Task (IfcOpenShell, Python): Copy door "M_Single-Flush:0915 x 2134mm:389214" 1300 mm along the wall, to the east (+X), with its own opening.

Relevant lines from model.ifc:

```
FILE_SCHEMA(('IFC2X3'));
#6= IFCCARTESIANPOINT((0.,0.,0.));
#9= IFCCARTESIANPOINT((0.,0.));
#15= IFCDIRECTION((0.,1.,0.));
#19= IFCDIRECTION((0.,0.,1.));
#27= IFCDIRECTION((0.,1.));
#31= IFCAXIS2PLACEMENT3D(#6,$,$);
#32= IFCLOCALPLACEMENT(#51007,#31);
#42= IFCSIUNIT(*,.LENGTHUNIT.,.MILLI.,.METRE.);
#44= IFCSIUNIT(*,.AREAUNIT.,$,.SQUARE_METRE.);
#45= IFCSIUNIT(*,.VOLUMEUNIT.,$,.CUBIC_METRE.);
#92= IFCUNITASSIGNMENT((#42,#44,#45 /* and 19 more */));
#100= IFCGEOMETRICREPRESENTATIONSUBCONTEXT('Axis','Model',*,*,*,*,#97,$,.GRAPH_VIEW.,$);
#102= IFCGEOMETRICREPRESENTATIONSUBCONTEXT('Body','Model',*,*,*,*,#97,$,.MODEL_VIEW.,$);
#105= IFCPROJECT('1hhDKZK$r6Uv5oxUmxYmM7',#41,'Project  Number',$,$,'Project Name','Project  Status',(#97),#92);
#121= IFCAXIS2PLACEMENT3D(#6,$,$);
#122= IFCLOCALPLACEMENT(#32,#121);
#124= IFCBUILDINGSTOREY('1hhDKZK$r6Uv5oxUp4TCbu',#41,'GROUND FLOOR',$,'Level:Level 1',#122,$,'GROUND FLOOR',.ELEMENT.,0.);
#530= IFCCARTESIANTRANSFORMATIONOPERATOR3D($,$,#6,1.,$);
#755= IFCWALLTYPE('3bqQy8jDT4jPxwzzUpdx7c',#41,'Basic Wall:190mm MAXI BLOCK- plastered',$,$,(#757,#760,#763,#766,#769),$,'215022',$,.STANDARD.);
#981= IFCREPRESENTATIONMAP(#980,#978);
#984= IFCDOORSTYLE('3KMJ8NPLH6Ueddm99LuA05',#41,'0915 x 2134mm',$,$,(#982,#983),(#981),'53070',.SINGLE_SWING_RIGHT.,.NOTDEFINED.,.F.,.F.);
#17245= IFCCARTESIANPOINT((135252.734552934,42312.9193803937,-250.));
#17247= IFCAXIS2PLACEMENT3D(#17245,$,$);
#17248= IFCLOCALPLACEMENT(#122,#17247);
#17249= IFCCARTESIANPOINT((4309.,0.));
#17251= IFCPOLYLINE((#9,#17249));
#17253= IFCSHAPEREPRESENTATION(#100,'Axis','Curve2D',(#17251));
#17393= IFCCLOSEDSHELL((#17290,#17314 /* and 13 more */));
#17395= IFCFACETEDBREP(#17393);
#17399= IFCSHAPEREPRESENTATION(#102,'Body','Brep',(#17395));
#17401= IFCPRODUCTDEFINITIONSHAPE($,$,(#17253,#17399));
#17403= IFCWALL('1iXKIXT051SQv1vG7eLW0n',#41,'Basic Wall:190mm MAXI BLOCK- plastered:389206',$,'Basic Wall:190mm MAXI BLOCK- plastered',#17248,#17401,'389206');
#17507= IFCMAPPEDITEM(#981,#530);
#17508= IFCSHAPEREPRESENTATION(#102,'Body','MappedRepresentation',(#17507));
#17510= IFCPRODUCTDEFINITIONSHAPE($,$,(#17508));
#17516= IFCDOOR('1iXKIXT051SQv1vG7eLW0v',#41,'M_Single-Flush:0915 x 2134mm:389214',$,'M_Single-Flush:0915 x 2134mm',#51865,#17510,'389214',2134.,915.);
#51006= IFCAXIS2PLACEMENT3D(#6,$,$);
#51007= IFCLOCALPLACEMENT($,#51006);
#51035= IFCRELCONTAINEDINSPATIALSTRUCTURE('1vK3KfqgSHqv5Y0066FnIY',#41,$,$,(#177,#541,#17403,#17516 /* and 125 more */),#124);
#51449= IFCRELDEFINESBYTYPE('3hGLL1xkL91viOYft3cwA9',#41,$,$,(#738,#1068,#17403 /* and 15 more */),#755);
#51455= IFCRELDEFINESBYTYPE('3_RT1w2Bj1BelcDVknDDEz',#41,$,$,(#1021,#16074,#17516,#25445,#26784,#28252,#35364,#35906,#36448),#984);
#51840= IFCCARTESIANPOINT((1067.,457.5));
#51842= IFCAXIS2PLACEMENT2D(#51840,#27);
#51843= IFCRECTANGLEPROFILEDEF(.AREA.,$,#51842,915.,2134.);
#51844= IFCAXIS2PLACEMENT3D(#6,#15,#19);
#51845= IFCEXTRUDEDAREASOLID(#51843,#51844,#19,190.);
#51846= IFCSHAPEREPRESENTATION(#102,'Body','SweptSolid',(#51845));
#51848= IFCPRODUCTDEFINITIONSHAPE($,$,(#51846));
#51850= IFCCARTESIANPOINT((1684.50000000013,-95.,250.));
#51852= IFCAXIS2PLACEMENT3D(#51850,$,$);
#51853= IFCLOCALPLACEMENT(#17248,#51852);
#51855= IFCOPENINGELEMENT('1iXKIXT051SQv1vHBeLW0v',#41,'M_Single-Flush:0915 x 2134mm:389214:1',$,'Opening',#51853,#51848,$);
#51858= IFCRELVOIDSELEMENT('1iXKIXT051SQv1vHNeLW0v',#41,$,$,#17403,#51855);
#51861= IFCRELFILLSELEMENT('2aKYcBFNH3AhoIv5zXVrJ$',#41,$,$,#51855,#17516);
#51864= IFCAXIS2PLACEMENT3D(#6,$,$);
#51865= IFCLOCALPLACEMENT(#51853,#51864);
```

```python
import ifcopenshell
import ifcopenshell.api.feature
import ifcopenshell.api.geometry
import ifcopenshell.api.root
import ifcopenshell.geom
import ifcopenshell.util.element
import ifcopenshell.util.placement
import ifcopenshell.util.shape
import ifcopenshell.util.unit

model = ifcopenshell.open("model.ifc")
unit_scale = ifcopenshell.util.unit.calculate_unit_scale(model)
settings = ifcopenshell.geom.settings()


def volume(element):
    """Net volume in cubic metres, openings subtracted."""
    shape = ifcopenshell.geom.create_shape(settings, element)
    return ifcopenshell.util.shape.get_volume(shape.geometry)


def reuse_history(source, copy):
    """copy_class also copies each property set's owner history, people and application; keep the originals."""
    for rel in copy.IsDefinedBy:
        if rel.is_a("IfcRelDefinesByProperties") and (history := rel.RelatingPropertyDefinition.OwnerHistory):
            rel.RelatingPropertyDefinition.OwnerHistory = source.OwnerHistory
            ifcopenshell.util.element.remove_deep2(model, history)


door = model.by_guid("1iXKIXT051SQv1vG7eLW0v")
opening = door.FillsVoids[0].RelatingOpeningElement
wall = opening.VoidsElements[0].RelatingBuildingElement
before = volume(wall)
shift = ifcopenshell.util.placement.get_local_placement(wall.ObjectPlacement)[:3, 0] * 1.3 / unit_scale

# copy_class copies the void relationship, type, container and properties, but no geometry.
new_opening = ifcopenshell.api.root.copy_class(model, product=opening)
new_opening.Representation = ifcopenshell.util.element.copy_deep(
    model, opening.Representation, exclude=["IfcGeometricRepresentationContext", "IfcRepresentationMap"]
)
new_opening.Name = "M_Single-Flush:0915 x 2134mm"
new_door = ifcopenshell.api.root.copy_class(model, product=door)
new_door.Representation = ifcopenshell.util.element.copy_deep(
    model, door.Representation, exclude=["IfcGeometricRepresentationContext", "IfcRepresentationMap"]
)
new_door.Name = "M_Single-Flush:0915 x 2134mm"
new_door.Tag = None
reuse_history(door, new_door)
fills = ifcopenshell.api.feature.add_filling(model, opening=new_opening, element=new_door)
fills.OwnerHistory = new_door.OwnerHistory  # required in IFC2X3

for old, new in ((opening, new_opening), (door, new_door)):
    matrix = ifcopenshell.util.placement.get_local_placement(old.ObjectPlacement)
    matrix[:3, 3] += shift
    ifcopenshell.api.geometry.edit_object_placement(model, product=new, matrix=matrix, is_si=False)

after = volume(wall)

print(f"wall volume {before:.3f} -> {after:.3f} m3")

model.write("model-out.ifc")
```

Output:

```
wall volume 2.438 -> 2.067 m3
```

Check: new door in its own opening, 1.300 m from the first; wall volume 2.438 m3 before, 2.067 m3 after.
